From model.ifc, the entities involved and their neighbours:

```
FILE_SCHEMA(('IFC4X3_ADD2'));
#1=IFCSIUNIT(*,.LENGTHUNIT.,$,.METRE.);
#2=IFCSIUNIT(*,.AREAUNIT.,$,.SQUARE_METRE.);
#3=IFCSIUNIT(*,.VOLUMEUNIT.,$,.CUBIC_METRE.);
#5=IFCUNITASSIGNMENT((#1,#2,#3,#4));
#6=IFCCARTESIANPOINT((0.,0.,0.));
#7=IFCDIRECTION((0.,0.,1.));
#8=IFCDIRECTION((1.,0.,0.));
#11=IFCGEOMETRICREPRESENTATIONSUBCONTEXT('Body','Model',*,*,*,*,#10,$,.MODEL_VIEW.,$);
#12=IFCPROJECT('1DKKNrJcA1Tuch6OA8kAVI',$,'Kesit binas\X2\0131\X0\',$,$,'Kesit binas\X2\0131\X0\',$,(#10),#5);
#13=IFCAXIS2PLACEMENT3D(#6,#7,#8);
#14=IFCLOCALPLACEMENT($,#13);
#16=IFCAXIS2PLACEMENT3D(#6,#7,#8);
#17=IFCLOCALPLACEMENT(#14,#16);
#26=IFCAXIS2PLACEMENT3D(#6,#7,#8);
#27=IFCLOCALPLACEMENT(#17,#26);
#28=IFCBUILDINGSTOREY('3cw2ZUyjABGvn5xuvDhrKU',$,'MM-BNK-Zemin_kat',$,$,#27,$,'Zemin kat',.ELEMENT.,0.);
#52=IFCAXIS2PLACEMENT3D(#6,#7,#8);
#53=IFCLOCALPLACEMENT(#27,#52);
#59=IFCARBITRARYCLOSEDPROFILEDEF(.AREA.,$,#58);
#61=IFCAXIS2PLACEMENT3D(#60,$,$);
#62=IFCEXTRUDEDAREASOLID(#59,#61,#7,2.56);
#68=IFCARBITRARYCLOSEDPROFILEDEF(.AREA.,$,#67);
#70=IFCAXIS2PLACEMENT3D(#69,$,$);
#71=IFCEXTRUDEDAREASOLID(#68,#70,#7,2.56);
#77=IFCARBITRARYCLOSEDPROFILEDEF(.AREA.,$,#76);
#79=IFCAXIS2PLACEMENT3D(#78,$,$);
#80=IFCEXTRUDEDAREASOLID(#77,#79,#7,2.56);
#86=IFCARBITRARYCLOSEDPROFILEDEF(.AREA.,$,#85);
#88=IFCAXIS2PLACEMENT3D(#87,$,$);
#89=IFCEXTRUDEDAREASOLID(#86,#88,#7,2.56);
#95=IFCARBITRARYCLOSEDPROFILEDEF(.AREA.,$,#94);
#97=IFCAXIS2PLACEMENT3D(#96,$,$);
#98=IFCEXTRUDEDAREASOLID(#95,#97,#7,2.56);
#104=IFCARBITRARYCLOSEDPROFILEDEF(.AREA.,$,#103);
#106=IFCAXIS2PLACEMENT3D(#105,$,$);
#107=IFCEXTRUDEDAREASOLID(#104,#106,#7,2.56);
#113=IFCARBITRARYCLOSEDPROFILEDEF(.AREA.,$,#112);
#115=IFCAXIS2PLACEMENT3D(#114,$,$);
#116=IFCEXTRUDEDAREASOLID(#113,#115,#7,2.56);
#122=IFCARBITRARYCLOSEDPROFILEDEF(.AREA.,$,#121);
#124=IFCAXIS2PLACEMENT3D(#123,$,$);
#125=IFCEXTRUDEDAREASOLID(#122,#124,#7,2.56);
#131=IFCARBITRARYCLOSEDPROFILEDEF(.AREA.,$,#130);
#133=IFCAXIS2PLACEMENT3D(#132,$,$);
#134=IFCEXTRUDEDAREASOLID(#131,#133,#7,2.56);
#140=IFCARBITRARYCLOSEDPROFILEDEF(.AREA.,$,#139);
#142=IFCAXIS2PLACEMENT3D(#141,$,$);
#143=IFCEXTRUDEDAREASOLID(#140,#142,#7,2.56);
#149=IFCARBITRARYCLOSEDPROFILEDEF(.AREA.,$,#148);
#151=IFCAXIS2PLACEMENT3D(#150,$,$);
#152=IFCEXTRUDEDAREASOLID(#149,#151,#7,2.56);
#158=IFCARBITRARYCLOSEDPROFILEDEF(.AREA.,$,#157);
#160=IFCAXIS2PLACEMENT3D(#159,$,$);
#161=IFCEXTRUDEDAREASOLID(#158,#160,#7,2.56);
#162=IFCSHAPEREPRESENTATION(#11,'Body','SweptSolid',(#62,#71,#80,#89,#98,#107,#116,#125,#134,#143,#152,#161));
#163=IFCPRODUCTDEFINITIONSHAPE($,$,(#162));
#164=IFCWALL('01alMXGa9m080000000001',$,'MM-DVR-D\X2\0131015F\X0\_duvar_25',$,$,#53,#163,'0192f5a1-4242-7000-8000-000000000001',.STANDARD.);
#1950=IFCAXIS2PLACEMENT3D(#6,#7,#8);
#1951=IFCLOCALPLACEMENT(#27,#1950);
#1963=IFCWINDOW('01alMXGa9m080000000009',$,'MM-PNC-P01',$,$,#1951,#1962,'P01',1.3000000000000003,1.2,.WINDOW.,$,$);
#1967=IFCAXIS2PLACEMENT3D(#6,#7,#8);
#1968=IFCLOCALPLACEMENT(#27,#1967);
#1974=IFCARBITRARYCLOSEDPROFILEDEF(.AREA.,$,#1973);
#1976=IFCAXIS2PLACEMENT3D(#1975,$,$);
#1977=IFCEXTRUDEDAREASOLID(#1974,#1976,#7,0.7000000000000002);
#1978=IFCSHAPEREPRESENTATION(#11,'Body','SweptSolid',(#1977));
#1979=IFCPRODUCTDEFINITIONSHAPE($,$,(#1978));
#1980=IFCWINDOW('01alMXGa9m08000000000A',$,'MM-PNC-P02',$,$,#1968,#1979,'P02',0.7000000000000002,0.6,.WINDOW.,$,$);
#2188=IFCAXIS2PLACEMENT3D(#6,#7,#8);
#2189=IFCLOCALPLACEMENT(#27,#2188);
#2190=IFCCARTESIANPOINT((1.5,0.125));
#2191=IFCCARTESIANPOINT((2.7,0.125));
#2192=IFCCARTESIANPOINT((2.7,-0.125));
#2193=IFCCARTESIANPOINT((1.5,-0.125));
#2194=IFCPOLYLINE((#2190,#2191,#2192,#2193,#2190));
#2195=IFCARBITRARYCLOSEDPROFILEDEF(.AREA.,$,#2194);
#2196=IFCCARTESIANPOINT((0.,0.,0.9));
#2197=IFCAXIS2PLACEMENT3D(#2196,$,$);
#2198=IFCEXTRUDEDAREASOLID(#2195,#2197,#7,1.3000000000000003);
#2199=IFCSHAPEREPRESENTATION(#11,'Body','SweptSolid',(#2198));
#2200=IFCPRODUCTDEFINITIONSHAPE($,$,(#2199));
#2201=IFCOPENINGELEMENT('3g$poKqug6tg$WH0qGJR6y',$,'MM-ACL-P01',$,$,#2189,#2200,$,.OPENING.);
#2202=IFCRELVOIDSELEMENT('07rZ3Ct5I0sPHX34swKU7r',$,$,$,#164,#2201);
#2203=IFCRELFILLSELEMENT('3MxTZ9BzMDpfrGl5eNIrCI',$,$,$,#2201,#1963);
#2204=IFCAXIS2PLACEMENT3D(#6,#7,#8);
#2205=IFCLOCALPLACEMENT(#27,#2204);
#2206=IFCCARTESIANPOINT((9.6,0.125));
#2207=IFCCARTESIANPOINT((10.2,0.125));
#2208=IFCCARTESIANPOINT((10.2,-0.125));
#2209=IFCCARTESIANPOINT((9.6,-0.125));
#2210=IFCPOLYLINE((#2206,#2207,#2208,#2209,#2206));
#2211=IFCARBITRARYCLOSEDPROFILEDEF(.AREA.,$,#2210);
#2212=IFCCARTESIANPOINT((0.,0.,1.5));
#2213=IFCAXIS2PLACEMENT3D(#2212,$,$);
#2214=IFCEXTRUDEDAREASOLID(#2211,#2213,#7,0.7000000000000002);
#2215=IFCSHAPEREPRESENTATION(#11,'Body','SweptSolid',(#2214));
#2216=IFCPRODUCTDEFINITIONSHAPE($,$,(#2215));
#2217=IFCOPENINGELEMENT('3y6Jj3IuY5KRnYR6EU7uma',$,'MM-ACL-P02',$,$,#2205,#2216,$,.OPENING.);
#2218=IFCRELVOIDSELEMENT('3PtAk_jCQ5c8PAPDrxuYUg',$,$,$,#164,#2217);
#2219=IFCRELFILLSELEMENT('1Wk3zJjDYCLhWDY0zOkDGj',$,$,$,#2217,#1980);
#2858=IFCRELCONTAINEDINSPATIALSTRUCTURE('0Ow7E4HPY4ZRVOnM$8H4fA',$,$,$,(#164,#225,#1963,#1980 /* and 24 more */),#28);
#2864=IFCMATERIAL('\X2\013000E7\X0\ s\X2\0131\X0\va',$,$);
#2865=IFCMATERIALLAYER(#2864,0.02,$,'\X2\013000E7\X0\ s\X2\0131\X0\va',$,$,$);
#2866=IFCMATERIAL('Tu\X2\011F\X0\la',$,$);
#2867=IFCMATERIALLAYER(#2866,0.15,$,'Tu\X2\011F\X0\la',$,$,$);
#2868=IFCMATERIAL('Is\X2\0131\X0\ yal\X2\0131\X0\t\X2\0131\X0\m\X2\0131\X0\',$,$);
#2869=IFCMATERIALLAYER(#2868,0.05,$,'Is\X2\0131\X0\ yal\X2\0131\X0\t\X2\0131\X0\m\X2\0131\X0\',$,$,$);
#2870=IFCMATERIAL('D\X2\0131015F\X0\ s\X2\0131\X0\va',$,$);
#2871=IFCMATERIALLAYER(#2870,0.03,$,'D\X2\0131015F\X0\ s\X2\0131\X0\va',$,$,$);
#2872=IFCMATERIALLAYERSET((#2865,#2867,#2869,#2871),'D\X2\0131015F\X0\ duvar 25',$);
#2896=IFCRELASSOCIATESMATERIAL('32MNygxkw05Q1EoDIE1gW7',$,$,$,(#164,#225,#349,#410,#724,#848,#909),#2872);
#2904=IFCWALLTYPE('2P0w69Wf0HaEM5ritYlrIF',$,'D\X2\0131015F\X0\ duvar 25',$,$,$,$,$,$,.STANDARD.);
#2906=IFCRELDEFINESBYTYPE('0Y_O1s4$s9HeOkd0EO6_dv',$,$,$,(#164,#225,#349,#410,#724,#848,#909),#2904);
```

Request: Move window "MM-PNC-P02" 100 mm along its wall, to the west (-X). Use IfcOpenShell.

```python
import ifcopenshell
import ifcopenshell.api.geometry
import ifcopenshell.util.placement
import ifcopenshell.util.unit

model = ifcopenshell.open("model.ifc")
unit_scale = ifcopenshell.util.unit.calculate_unit_scale(model)

window = model.by_guid("01alMXGa9m08000000000A")
opening = window.FillsVoids[0].RelatingOpeningElement
wall = opening.VoidsElements[0].RelatingBuildingElement

wall_matrix = ifcopenshell.util.placement.get_local_placement(wall.ObjectPlacement)
shift = wall_matrix[:3, 0] * -0.1 / unit_scale
before = ifcopenshell.util.placement.get_local_placement(window.ObjectPlacement)[:3, 3].copy()

# The window is not placed relative to its opening, so move both.
for product in (opening, window):
    matrix = ifcopenshell.util.placement.get_local_placement(product.ObjectPlacement)
    matrix[:3, 3] += shift
    ifcopenshell.api.geometry.edit_object_placement(model, product=product, matrix=matrix, is_si=False)

after = ifcopenshell.util.placement.get_local_placement(window.ObjectPlacement)[:3, 3]
print("window moved by", (after - before).round(3) + 0.0)

model.write("model-out.ifc")
```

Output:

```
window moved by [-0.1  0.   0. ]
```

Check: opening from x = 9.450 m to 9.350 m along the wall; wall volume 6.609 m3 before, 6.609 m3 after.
